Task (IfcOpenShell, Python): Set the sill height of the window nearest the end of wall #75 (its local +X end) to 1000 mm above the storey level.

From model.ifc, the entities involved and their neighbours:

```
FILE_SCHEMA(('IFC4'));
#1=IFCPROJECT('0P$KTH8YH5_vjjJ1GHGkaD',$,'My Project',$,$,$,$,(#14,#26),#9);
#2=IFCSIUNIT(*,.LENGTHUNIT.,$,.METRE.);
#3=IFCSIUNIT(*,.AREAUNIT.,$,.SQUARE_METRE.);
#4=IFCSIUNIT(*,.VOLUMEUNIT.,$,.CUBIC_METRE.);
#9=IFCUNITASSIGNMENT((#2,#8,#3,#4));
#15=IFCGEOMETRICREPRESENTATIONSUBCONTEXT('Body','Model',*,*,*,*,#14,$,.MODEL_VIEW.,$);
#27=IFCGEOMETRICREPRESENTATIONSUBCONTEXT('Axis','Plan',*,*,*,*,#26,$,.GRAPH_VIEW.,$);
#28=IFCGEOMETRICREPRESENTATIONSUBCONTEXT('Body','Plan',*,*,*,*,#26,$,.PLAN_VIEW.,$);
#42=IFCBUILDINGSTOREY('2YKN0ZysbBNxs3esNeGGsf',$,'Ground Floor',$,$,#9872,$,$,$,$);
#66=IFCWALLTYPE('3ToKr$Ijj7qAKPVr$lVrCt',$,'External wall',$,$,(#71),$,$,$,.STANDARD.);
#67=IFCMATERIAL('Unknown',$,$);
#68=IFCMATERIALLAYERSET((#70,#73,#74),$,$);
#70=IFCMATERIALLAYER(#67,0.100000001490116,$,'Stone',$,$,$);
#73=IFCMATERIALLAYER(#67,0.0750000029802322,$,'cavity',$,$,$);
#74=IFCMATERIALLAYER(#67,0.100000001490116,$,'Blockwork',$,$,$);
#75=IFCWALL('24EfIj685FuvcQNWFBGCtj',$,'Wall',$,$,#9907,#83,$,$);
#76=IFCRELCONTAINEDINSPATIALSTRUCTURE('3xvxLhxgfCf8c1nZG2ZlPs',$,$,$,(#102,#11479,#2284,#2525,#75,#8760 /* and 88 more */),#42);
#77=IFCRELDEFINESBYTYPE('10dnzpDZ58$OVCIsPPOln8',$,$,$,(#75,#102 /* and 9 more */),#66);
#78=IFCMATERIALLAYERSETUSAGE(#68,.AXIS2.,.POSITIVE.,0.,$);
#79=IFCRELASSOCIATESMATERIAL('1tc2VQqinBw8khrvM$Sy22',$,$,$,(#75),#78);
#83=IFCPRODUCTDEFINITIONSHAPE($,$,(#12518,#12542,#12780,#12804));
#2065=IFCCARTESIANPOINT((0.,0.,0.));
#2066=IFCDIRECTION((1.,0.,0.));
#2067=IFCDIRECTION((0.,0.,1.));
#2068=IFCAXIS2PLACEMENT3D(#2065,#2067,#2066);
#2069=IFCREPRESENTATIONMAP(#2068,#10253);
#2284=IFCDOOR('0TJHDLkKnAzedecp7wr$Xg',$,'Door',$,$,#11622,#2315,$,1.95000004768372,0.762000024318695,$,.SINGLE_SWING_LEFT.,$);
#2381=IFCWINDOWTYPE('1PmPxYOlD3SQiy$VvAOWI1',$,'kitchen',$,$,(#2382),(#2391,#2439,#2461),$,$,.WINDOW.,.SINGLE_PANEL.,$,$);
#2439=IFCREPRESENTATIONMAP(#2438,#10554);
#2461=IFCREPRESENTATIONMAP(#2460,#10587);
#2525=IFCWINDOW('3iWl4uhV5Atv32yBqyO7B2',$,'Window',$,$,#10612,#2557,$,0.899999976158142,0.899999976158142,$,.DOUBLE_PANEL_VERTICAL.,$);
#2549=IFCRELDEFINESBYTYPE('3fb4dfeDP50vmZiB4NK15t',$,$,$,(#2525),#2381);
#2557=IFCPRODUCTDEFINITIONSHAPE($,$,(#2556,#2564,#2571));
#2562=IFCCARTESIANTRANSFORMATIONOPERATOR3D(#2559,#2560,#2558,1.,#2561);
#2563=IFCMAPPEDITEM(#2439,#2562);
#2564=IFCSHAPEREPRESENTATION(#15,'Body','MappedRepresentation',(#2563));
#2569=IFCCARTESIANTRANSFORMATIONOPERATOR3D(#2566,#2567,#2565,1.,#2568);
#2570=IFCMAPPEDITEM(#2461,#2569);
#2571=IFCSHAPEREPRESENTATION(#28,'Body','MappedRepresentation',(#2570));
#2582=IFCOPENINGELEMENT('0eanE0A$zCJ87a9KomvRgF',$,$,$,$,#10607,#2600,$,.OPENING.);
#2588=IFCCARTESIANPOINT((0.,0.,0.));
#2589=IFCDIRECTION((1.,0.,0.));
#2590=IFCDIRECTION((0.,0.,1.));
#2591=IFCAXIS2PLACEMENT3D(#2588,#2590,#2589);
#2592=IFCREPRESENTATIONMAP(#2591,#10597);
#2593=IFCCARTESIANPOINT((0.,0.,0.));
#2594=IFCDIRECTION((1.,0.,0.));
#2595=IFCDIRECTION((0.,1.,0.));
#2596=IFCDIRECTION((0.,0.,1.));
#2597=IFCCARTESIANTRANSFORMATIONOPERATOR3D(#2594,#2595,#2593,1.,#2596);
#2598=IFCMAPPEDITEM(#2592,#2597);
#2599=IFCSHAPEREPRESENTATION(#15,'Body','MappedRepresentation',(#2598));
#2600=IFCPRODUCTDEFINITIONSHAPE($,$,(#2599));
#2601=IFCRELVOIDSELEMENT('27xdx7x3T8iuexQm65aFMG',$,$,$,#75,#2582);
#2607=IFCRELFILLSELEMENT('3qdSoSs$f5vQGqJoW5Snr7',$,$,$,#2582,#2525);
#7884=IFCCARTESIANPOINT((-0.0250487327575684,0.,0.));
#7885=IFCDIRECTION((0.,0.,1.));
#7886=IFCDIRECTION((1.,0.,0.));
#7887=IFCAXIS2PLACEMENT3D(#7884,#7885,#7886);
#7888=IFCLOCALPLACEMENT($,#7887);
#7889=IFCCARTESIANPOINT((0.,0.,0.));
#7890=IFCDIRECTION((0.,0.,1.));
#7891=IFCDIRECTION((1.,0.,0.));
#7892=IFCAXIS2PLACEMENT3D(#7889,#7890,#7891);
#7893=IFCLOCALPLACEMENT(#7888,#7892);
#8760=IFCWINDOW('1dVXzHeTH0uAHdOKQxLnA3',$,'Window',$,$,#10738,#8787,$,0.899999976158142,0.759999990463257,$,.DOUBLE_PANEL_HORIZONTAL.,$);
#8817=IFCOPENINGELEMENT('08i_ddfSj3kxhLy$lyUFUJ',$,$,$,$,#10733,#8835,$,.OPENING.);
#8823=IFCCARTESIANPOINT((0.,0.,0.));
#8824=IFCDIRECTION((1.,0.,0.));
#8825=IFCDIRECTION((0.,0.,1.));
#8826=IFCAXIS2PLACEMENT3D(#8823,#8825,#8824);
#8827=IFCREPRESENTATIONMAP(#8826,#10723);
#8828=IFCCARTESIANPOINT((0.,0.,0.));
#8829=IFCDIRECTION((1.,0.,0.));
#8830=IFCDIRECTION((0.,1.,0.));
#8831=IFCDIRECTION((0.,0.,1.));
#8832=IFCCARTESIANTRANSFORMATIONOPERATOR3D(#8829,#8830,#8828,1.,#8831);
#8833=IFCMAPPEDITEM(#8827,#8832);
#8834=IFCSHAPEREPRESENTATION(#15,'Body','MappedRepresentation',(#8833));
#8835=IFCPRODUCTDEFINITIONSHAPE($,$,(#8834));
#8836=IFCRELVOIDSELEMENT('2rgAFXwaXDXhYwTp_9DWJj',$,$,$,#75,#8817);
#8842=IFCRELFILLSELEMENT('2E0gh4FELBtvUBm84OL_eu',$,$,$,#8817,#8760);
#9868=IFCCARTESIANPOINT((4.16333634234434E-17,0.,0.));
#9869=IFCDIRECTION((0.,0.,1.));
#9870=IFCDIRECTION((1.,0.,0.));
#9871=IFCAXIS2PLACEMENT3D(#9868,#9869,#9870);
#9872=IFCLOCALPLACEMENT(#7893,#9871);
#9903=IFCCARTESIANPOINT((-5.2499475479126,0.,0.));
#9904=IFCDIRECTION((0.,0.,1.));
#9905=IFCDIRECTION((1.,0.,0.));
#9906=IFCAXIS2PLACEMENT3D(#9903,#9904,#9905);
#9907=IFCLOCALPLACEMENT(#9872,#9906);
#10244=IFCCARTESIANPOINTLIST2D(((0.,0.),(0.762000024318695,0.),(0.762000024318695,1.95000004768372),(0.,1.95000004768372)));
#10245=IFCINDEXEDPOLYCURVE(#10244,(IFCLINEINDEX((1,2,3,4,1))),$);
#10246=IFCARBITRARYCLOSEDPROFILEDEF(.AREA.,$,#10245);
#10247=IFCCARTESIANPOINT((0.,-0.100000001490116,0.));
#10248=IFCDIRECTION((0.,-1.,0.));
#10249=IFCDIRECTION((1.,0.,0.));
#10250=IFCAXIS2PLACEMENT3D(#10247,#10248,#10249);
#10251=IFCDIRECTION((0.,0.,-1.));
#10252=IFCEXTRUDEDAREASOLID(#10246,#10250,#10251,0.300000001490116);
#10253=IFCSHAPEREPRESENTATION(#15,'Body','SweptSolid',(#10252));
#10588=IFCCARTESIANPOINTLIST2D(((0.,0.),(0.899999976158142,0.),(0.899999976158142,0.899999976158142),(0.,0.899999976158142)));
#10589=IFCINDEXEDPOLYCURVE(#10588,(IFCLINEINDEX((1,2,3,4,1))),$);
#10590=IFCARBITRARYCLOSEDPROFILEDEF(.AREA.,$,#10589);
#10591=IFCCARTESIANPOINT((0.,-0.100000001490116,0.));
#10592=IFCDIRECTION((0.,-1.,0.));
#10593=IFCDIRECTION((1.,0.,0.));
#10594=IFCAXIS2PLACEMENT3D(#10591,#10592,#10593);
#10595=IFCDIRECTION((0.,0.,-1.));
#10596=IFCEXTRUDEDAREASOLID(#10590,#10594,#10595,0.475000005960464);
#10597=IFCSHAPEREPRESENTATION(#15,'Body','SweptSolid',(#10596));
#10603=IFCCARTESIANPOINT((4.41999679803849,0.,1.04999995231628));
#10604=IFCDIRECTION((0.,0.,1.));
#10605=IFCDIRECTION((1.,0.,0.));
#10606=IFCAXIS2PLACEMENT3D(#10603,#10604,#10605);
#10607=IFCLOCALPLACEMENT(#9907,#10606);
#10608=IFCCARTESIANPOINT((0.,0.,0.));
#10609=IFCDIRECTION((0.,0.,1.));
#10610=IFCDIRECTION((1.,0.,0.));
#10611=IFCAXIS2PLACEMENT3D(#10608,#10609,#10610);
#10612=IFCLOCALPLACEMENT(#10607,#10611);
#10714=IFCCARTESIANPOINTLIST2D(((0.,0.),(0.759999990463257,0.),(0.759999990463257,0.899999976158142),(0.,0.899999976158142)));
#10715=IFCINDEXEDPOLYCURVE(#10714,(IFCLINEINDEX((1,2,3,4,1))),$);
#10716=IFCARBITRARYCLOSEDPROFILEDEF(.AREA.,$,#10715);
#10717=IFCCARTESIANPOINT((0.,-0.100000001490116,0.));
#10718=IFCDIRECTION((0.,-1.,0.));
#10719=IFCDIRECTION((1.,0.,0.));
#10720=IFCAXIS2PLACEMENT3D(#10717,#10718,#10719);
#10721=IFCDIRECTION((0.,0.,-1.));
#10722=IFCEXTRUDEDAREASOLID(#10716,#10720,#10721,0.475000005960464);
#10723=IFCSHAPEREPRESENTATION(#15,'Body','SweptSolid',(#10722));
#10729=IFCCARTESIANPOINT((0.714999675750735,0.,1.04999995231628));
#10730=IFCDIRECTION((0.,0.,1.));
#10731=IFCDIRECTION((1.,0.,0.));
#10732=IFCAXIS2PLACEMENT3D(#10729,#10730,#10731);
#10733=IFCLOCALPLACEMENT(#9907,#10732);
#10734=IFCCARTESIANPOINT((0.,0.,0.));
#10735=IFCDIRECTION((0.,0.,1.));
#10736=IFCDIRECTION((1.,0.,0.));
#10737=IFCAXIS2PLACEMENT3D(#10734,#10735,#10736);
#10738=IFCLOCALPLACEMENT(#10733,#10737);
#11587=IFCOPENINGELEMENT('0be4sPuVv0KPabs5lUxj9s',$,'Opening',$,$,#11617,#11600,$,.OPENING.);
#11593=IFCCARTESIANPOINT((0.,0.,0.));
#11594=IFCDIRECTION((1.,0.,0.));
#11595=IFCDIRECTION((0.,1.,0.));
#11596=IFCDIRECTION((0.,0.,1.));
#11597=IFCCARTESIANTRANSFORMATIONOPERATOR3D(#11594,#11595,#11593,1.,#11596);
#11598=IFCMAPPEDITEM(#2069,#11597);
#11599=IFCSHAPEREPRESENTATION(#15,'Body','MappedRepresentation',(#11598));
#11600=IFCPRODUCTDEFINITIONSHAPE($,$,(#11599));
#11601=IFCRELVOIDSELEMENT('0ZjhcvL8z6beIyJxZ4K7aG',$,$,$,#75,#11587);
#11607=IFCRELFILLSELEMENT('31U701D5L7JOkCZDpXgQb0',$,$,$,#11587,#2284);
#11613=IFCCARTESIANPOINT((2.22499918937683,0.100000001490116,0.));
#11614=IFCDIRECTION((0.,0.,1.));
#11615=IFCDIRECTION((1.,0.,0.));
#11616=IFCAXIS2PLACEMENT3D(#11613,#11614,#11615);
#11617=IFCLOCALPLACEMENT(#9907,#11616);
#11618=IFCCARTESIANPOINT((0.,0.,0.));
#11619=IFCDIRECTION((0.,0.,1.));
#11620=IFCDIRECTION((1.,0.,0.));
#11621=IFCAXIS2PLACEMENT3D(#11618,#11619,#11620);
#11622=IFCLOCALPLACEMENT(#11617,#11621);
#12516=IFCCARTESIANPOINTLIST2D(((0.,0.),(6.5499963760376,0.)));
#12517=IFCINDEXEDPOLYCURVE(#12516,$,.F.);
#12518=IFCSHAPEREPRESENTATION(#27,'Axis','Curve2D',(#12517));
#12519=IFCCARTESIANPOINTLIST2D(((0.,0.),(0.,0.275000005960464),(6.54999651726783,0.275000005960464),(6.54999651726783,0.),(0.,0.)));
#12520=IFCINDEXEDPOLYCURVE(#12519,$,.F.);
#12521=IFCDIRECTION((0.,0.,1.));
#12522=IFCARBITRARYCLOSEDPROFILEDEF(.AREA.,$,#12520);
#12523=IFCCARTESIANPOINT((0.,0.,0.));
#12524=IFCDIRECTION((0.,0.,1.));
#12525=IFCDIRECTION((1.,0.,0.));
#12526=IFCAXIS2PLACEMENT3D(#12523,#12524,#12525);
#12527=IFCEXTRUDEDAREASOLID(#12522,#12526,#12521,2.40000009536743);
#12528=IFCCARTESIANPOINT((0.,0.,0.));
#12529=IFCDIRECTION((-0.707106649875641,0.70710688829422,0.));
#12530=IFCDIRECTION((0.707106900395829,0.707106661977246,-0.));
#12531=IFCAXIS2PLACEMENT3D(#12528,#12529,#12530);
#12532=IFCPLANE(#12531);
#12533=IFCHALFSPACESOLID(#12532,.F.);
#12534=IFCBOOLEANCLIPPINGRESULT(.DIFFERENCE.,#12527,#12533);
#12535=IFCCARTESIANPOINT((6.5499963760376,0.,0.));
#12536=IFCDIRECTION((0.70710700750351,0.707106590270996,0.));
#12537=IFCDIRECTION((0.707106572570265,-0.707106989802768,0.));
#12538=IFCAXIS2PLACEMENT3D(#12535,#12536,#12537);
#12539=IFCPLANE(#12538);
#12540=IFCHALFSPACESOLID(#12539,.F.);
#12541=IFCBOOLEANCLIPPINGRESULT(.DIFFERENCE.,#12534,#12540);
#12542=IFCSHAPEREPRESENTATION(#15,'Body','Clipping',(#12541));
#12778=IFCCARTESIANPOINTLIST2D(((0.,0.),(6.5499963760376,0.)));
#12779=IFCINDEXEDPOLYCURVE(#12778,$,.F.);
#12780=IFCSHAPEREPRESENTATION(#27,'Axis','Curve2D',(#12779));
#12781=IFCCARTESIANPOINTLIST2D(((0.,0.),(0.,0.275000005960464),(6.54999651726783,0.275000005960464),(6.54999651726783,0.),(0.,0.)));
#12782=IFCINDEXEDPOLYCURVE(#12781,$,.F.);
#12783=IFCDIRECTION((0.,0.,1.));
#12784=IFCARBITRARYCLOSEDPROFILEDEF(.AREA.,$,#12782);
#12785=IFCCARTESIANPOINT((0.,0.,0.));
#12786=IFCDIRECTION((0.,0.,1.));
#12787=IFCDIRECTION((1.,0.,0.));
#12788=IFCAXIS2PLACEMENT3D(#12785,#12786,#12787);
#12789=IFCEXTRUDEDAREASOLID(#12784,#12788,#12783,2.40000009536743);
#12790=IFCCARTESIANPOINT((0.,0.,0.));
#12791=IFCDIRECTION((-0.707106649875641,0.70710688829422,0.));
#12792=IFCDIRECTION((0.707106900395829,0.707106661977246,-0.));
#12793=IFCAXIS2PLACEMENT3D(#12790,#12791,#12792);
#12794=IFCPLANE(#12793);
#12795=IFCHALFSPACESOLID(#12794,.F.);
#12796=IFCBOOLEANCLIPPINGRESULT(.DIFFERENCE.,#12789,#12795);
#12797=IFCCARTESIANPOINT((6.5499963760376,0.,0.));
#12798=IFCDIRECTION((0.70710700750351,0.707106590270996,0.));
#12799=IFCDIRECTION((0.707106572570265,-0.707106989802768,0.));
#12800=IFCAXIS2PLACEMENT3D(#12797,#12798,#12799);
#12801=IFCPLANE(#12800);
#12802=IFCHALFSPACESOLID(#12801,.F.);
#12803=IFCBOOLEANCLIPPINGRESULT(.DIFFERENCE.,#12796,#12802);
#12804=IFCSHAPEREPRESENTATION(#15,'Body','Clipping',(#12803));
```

```python
import numpy as np
import ifcopenshell
import ifcopenshell.api.geometry
import ifcopenshell.geom
import ifcopenshell.util.element
import ifcopenshell.util.placement
import ifcopenshell.util.shape
import ifcopenshell.util.unit

model = ifcopenshell.open("model.ifc")
unit_scale = ifcopenshell.util.unit.calculate_unit_scale(model)

window = model.by_guid("3iWl4uhV5Atv32yBqyO7B2")
opening = window.FillsVoids[0].RelatingOpeningElement
storey = ifcopenshell.util.element.get_container(window, ifc_class="IfcBuildingStorey")
level = ifcopenshell.util.placement.get_local_placement(storey.ObjectPlacement)[2, 3]

# The opening's origin need not be at the sill, so measure its lowest point.
shape = ifcopenshell.geom.create_shape(ifcopenshell.geom.settings(), opening)
bottom = ifcopenshell.util.shape.get_shape_bottom_elevation(shape, shape.geometry) / unit_scale
dz = level + 1.0 - bottom

shift = np.array([0.0, 0.0, dz])
# The window is placed relative to its opening, so it follows when the opening moves.
matrix = ifcopenshell.util.placement.get_local_placement(opening.ObjectPlacement)
matrix[:3, 3] += shift
ifcopenshell.api.geometry.edit_object_placement(
    model, product=opening, matrix=matrix, is_si=False, should_transform_children=True
)

print(f"moved by {dz * unit_scale:+.3f} m")

model.write("model_v2.ifc")
```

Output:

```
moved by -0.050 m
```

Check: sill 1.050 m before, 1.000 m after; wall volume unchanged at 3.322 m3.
